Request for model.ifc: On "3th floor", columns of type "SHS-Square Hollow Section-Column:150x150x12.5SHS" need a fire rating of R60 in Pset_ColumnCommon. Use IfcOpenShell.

First a look at what the model holds.

```python
import ifcopenshell
import ifcopenshell.util.element

model = ifcopenshell.open("model.ifc")
print(model.schema)
storey = next(s for s in model.by_type("IfcBuildingStorey") if s.Name == "3th floor")
columns = [e for e in ifcopenshell.util.element.get_decomposition(storey) if e.is_a("IfcColumn")]
seen = {}
for e in columns:
    element_type = ifcopenshell.util.element.get_type(e)
    key = (element_type.Name if element_type != e and element_type else None, ifcopenshell.util.element.get_pset(e, "Pset_ColumnCommon", "FireRating"))
    seen[key] = seen.get(key, 0) + 1
for (name, value), count in sorted(seen.items(), key=str):
    print(count, "x", name, "|", value)
```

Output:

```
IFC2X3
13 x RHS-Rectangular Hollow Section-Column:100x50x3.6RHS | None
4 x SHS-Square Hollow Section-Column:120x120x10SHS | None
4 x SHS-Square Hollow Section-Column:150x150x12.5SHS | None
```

```python
import ifcopenshell
import ifcopenshell.api.pset
import ifcopenshell.util.element

model = ifcopenshell.open("model.ifc")

storey = next(s for s in model.by_type("IfcBuildingStorey") if s.Name == "3th floor")
columns = [e for e in ifcopenshell.util.element.get_decomposition(storey) if e.is_a("IfcColumn")]

count = 0
for e in columns:
    element_type = ifcopenshell.util.element.get_type(e)
    if element_type in (None, e) or element_type.Name != "SHS-Square Hollow Section-Column:150x150x12.5SHS":
        continue
    # add_pset returns the element's existing set when there is one.
    pset = ifcopenshell.api.pset.add_pset(model, product=e, name="Pset_ColumnCommon")
    ifcopenshell.api.pset.edit_pset(model, pset=pset, properties={"FireRating": "R60"})
    count += 1

print(count, "columns updated")

model.write("model-out.ifc")
```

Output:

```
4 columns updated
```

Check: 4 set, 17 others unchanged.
